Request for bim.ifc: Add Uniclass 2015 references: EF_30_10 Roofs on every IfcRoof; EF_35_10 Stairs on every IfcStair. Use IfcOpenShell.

First a look at what the model holds.

```python
import ifcopenshell

model = ifcopenshell.open("bim.ifc")
print(model.schema)
print("classifications:", [c.Name for c in model.by_type("IfcClassification")])
for ifc_class in ("IfcDoor", "IfcRoof", "IfcStair", "IfcWall", "IfcWindow"):
    print(ifc_class, len(model.by_type(ifc_class)))
```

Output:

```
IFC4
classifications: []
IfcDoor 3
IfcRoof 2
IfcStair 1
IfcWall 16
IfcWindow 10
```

```python
import ifcopenshell
import ifcopenshell.api.classification

model = ifcopenshell.open("bim.ifc")

system = ifcopenshell.api.classification.add_classification(model, classification="Uniclass 2015")

codes = {
    "IfcRoof": ("EF_30_10", "Roofs"),
    "IfcStair": ("EF_35_10", "Stairs"),
}
for ifc_class, (code, name) in codes.items():
    products = model.by_type(ifc_class)
    ifcopenshell.api.classification.add_reference(
        model, products=products, classification=system, identification=code, name=name
    )
    print(code, len(products))

model.write("bim_rev.ifc")
```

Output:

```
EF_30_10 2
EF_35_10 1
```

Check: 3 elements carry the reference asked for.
